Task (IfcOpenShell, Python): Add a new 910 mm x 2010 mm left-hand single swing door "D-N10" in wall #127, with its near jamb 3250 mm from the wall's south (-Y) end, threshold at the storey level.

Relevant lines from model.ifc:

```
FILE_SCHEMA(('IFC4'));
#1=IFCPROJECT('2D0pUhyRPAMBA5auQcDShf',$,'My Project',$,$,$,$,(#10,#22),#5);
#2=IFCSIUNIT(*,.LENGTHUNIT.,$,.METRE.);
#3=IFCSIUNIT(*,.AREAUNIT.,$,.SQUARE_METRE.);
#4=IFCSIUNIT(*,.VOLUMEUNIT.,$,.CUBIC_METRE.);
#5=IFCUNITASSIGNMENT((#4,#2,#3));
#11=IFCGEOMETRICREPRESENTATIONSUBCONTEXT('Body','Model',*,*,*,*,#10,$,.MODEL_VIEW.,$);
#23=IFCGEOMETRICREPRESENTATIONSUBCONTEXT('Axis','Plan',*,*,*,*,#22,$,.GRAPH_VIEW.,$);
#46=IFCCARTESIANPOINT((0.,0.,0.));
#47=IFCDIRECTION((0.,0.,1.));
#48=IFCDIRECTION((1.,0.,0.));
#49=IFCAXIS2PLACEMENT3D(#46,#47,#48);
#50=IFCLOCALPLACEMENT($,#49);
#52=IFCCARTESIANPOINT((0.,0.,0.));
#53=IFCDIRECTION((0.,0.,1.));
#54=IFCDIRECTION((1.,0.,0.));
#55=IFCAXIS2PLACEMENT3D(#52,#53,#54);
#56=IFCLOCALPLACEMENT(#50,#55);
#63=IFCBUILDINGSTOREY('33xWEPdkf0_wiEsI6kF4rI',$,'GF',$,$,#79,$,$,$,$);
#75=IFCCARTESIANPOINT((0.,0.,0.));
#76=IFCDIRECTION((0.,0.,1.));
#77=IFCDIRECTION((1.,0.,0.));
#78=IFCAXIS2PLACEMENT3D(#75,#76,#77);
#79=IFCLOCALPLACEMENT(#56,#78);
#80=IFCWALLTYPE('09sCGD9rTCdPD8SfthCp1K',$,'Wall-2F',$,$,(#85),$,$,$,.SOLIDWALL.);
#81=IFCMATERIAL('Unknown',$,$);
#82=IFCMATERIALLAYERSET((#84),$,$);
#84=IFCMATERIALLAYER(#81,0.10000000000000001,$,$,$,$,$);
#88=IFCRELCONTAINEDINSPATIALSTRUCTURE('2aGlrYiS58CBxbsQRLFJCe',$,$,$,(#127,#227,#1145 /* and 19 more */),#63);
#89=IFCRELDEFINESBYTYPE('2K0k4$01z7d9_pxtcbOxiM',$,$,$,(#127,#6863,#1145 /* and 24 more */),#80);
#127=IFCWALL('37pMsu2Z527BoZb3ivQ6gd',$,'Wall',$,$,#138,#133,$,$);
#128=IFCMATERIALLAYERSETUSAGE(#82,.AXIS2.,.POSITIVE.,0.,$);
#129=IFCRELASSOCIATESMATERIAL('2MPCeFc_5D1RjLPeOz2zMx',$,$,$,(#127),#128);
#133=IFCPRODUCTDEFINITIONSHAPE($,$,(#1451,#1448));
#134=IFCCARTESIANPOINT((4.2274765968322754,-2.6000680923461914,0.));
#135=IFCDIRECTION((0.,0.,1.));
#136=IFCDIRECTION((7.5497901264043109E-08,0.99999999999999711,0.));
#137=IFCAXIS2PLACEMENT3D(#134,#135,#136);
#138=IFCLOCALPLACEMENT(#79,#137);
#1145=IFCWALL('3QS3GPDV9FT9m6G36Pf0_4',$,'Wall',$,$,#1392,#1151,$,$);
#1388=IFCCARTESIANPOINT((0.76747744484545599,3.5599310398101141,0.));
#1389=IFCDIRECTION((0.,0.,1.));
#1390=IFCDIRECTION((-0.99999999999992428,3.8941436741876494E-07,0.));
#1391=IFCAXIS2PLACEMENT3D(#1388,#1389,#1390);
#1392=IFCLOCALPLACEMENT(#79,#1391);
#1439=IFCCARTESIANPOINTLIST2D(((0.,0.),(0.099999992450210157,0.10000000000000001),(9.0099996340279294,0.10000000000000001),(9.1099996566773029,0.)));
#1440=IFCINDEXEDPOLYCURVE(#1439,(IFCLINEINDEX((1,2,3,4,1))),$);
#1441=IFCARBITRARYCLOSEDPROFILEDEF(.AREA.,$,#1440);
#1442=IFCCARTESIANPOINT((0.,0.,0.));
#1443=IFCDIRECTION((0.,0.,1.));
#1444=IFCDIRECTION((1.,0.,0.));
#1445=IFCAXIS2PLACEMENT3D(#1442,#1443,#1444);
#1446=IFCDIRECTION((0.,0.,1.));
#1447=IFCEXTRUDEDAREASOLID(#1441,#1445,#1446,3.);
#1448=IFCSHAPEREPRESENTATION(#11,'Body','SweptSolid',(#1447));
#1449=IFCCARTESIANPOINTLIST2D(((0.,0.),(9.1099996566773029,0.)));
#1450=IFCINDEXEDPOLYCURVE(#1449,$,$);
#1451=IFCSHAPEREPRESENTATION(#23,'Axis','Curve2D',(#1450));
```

```python
import numpy as np
import ifcopenshell
import ifcopenshell.api.feature
import ifcopenshell.api.geometry
import ifcopenshell.api.root
import ifcopenshell.api.spatial
import ifcopenshell.geom
import ifcopenshell.util.element
import ifcopenshell.util.placement
import ifcopenshell.util.representation
import ifcopenshell.util.shape
import ifcopenshell.util.unit

model = ifcopenshell.open("model.ifc")
unit_scale = ifcopenshell.util.unit.calculate_unit_scale(model)
settings = ifcopenshell.geom.settings()


def volume(element):
    """Net volume in cubic metres, openings subtracted."""
    shape = ifcopenshell.geom.create_shape(settings, element)
    return ifcopenshell.util.shape.get_volume(shape.geometry)


wall = model.by_id(127)
storey = ifcopenshell.util.element.get_container(wall, ifc_class="IfcBuildingStorey")
context = ifcopenshell.util.representation.get_context(model, "Model", "Body", "MODEL_VIEW")
before = volume(wall)

width, height, from_end, sill = 0.91, 2.01, 3.25, 0.0  # metres

# The wall runs along its own X axis, and the end named is its -X end.
wall_shape = ifcopenshell.geom.create_shape(settings, wall)
x, y, z = ifcopenshell.util.shape.get_vertices(wall_shape.geometry).T
start = x.min() + from_end
face, thickness = float(y.min()), float(y.max() - y.min())
wall_matrix = ifcopenshell.util.placement.get_local_placement(wall.ObjectPlacement)
level = ifcopenshell.util.placement.get_local_placement(storey.ObjectPlacement)[2, 3]


def in_wall(x, y):
    """Placement at x, y metres in the wall's axes, at sill height."""
    matrix = wall_matrix.copy()
    matrix[:, 3] = wall_matrix @ np.array([x / unit_scale, y / unit_scale, 0.0, 1.0])
    matrix[2, 3] = level + sill / unit_scale
    return matrix


# Opening: a box that overshoots both wall faces by 50 mm.
opening = ifcopenshell.api.root.create_entity(model, ifc_class="IfcOpeningElement", predefined_type="OPENING")
box = ifcopenshell.api.geometry.add_wall_representation(
    model, context=context, length=width, height=height, thickness=thickness + 0.1
)
ifcopenshell.api.geometry.assign_representation(model, product=opening, representation=box)
ifcopenshell.api.geometry.edit_object_placement(model, product=opening, matrix=in_wall(start, face - 0.05), is_si=False)
ifcopenshell.api.feature.add_feature(model, feature=opening, element=wall)

door = ifcopenshell.api.root.create_entity(model, ifc_class="IfcDoor", name="D-N10", predefined_type="DOOR")
door.OverallWidth, door.OverallHeight = width / unit_scale, height / unit_scale
door.OperationType = "SINGLE_SWING_LEFT"
body = ifcopenshell.api.geometry.add_door_representation(
    model,
    context=context,
    overall_width=door.OverallWidth,
    overall_height=door.OverallHeight,
    operation_type="SINGLE_SWING_LEFT",
    lining_properties={"LiningDepth": thickness / unit_scale, "ThresholdDepth": thickness / unit_scale},
)
ifcopenshell.api.geometry.assign_representation(model, product=door, representation=body)
ifcopenshell.api.spatial.assign_container(model, products=[door], relating_structure=storey)
ifcopenshell.api.feature.add_filling(model, opening=opening, element=door)

# The lining spans the wall, so the door starts at the wall face.
ifcopenshell.api.geometry.edit_object_placement(model, product=door, matrix=in_wall(start, face), is_si=False)

after = volume(wall)

print(f"wall volume {before:.3f} -> {after:.3f} m3")

model.write("model_edited.ifc")
```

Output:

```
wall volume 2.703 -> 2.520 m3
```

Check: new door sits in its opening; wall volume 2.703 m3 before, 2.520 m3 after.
